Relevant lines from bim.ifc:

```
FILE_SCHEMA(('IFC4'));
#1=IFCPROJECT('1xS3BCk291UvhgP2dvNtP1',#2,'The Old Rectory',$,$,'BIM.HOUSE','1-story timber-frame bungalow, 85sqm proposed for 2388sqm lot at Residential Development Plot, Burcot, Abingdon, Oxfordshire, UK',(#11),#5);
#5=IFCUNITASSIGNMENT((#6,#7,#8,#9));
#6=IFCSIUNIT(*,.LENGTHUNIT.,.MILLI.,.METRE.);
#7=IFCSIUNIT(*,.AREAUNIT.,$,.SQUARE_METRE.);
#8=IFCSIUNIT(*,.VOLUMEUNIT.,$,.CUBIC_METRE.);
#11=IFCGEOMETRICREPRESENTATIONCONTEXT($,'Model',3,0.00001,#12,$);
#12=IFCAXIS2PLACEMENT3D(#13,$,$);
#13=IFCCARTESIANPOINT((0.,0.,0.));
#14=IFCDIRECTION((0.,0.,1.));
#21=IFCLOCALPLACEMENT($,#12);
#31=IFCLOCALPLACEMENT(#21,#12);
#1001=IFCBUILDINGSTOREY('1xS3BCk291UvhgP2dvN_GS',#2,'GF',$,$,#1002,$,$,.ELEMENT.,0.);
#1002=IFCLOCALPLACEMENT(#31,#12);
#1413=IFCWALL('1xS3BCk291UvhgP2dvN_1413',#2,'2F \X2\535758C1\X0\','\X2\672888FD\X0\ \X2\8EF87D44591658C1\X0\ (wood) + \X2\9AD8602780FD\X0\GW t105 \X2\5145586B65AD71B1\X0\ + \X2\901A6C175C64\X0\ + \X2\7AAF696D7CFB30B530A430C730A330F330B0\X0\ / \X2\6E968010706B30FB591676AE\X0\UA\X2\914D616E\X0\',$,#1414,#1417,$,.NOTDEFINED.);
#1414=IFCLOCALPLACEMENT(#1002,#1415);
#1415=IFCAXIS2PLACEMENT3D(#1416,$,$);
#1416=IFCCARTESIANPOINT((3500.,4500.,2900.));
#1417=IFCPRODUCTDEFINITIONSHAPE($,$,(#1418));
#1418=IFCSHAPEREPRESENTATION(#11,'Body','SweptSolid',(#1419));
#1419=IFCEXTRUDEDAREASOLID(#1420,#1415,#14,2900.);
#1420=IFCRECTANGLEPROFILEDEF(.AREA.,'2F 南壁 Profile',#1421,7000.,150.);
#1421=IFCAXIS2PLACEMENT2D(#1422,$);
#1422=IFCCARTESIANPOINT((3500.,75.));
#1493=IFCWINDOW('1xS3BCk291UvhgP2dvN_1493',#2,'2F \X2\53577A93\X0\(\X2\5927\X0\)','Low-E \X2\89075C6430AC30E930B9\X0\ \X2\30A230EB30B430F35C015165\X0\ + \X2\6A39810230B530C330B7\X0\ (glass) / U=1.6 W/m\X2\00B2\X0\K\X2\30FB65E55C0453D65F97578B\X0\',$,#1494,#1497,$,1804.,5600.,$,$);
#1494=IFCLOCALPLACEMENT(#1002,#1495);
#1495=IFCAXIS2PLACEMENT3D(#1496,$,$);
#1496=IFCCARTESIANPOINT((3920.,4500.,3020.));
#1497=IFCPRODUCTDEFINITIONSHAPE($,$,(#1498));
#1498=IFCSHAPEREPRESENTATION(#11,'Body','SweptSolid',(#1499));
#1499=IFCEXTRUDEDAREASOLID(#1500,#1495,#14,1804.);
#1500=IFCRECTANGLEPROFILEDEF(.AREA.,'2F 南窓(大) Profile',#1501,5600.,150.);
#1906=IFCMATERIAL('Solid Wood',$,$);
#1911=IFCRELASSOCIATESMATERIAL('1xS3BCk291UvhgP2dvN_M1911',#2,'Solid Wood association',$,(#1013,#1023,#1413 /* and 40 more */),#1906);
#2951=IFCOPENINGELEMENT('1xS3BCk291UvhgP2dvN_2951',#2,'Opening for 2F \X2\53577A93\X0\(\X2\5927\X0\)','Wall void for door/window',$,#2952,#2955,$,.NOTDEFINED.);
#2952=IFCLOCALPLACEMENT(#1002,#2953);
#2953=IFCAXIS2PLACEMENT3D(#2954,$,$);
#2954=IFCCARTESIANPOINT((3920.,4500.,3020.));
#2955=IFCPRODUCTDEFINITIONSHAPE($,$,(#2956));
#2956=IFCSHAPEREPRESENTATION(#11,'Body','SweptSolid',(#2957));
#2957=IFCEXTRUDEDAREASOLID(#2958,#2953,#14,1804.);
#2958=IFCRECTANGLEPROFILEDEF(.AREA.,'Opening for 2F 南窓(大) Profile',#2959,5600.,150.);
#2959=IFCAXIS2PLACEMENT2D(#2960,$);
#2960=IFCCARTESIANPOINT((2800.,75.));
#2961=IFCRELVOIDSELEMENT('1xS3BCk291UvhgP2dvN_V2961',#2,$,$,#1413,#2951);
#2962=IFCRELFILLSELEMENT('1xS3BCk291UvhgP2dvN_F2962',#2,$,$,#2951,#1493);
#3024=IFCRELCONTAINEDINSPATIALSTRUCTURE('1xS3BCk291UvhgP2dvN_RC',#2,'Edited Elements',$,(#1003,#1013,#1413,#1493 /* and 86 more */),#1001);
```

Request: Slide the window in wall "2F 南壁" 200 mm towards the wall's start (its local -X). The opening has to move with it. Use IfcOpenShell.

```python
import ifcopenshell
import ifcopenshell.api.geometry
import ifcopenshell.util.placement
import ifcopenshell.util.unit

model = ifcopenshell.open("bim.ifc")
unit_scale = ifcopenshell.util.unit.calculate_unit_scale(model)

window = model.by_guid("1xS3BCk291UvhgP2dvN_1493")
opening = window.FillsVoids[0].RelatingOpeningElement
wall = opening.VoidsElements[0].RelatingBuildingElement

wall_matrix = ifcopenshell.util.placement.get_local_placement(wall.ObjectPlacement)
shift = wall_matrix[:3, 0] * -0.2 / unit_scale
before = ifcopenshell.util.placement.get_local_placement(window.ObjectPlacement)[:3, 3].copy()

# The window is not placed relative to its opening, so move both.
for product in (opening, window):
    matrix = ifcopenshell.util.placement.get_local_placement(product.ObjectPlacement)
    matrix[:3, 3] += shift
    ifcopenshell.api.geometry.edit_object_placement(model, product=product, matrix=matrix, is_si=False)

after = ifcopenshell.util.placement.get_local_placement(window.ObjectPlacement)[:3, 3]
print("window moved by", (after - before).round(3) + 0.0)

model.write("bim_rev.ifc")
```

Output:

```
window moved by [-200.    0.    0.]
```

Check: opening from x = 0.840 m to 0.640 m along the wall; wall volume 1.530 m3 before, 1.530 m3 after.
